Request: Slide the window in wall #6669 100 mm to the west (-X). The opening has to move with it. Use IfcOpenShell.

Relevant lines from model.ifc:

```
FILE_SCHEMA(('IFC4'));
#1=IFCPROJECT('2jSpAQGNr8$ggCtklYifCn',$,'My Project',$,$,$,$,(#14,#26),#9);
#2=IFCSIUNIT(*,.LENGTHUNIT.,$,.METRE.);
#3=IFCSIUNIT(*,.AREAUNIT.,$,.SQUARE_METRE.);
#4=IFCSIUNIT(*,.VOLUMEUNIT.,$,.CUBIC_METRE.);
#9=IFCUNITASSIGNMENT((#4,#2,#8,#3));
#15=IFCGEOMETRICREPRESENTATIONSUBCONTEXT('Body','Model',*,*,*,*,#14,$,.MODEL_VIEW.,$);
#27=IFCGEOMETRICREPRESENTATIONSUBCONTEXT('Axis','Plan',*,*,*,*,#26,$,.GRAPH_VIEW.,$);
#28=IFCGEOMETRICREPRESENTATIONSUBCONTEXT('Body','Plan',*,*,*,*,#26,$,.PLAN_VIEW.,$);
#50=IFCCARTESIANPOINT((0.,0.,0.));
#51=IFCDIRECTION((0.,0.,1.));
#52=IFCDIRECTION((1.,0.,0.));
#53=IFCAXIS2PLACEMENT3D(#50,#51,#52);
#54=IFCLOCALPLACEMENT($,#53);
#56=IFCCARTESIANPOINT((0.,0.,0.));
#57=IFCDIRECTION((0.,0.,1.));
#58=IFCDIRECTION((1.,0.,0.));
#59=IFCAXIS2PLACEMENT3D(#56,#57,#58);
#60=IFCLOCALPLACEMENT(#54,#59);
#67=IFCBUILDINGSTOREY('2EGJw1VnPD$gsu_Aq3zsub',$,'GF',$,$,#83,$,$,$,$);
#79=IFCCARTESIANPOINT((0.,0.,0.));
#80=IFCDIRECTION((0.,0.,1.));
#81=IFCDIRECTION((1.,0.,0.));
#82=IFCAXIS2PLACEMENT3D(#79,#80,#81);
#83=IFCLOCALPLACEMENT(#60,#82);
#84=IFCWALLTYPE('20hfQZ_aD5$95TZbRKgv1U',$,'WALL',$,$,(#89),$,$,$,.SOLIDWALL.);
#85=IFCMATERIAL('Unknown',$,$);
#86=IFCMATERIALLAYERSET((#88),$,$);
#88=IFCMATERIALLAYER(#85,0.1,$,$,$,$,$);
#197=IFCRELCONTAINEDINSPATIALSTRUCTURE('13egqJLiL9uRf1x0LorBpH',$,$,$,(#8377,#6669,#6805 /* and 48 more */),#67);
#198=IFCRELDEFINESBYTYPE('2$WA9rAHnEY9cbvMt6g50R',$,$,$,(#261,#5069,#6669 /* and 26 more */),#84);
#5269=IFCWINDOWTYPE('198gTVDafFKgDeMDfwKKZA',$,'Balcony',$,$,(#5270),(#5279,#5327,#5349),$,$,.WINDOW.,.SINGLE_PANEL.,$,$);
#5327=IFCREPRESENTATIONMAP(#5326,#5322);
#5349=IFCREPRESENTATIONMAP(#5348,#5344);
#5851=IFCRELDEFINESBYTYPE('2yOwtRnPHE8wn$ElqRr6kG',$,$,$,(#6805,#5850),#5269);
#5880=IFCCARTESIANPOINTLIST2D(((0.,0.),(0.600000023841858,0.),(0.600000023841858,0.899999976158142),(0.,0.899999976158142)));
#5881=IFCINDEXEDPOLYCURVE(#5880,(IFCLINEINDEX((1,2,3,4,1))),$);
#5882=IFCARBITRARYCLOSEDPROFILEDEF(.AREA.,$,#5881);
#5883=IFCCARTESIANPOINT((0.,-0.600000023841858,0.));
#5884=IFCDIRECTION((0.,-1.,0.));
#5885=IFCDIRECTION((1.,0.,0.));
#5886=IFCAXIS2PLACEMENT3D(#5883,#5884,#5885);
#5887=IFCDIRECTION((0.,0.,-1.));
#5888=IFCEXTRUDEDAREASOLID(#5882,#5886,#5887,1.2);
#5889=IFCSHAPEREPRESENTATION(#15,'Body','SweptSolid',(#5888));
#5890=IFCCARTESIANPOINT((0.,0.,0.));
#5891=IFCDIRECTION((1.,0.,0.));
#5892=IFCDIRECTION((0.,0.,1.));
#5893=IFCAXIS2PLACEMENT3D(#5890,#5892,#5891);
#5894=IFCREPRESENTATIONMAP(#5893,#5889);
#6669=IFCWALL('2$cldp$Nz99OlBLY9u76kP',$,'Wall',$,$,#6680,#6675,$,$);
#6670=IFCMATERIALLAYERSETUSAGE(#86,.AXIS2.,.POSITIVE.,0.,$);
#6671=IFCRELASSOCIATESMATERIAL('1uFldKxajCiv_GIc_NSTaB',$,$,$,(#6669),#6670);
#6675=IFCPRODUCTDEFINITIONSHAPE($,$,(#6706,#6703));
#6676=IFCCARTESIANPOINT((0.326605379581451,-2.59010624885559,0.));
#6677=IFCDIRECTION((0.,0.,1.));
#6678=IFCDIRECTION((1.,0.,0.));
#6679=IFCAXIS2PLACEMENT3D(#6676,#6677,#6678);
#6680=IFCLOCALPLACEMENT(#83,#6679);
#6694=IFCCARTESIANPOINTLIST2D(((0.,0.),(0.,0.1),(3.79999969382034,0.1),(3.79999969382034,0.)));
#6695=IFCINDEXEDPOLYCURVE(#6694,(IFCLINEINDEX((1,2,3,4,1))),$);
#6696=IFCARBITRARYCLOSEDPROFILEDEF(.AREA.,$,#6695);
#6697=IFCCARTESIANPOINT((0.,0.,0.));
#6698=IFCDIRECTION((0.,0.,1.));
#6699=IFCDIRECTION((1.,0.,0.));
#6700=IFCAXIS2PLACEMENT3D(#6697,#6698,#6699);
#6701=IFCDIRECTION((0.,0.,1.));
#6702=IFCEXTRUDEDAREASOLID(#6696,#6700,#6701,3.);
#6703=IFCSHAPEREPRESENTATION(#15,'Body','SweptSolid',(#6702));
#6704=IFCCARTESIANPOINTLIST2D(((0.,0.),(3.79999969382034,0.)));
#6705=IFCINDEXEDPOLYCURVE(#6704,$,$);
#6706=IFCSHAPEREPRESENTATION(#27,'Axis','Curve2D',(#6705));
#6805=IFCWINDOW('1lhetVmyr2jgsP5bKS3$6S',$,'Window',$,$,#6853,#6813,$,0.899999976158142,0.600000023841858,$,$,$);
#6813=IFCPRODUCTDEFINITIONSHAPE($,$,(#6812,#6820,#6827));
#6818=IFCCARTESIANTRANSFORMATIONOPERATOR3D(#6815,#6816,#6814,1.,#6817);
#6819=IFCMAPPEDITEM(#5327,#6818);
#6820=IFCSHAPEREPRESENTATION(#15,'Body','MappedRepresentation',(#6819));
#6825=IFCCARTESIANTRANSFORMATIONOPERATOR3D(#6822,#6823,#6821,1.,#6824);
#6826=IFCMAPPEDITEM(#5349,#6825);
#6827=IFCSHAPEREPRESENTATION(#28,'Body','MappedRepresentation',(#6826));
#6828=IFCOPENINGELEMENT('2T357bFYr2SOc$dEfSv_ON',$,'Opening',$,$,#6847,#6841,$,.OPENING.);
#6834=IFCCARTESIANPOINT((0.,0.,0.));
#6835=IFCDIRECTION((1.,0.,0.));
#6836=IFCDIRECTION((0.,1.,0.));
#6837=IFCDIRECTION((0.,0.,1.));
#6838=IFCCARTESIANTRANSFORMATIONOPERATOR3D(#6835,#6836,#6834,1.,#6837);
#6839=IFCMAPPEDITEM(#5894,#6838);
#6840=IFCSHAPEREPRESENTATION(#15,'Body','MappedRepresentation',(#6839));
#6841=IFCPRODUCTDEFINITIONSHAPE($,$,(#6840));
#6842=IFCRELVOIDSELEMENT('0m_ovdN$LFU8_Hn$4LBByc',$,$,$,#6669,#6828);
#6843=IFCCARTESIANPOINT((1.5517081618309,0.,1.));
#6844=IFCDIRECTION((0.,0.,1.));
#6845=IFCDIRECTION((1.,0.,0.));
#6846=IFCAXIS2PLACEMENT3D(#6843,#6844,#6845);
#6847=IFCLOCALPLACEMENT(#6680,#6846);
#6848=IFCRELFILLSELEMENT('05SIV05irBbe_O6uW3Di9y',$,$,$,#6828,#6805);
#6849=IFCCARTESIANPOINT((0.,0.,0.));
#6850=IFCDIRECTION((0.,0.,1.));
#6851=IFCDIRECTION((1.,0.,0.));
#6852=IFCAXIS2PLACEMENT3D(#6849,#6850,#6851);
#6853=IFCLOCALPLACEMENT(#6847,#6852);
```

```python
import ifcopenshell
import ifcopenshell.api.geometry
import ifcopenshell.util.placement
import ifcopenshell.util.unit

model = ifcopenshell.open("model.ifc")
unit_scale = ifcopenshell.util.unit.calculate_unit_scale(model)

window = model.by_guid("1lhetVmyr2jgsP5bKS3$6S")
opening = window.FillsVoids[0].RelatingOpeningElement
wall = opening.VoidsElements[0].RelatingBuildingElement

wall_matrix = ifcopenshell.util.placement.get_local_placement(wall.ObjectPlacement)
shift = wall_matrix[:3, 0] * -0.1 / unit_scale
before = ifcopenshell.util.placement.get_local_placement(window.ObjectPlacement)[:3, 3].copy()

# The window is placed relative to its opening, so it follows when the opening moves.
matrix = ifcopenshell.util.placement.get_local_placement(opening.ObjectPlacement)
matrix[:3, 3] += shift
ifcopenshell.api.geometry.edit_object_placement(
    model, product=opening, matrix=matrix, is_si=False, should_transform_children=True
)

after = ifcopenshell.util.placement.get_local_placement(window.ObjectPlacement)[:3, 3]
print("window moved by", (after - before).round(3) + 0.0)

model.write("model_v2.ifc")
```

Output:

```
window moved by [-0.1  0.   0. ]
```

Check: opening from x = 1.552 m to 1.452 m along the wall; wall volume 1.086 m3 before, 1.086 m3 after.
